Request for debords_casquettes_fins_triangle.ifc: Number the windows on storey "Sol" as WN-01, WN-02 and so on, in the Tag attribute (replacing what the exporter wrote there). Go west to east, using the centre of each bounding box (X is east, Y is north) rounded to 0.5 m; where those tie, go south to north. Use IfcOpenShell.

First a look at what the model holds.

```python
import ifcopenshell
import ifcopenshell.util.element
import ifcopenshell.util.placement

model = ifcopenshell.open("debords_casquettes_fins_triangle.ifc")
print(model.schema)
storey = next(s for s in model.by_type("IfcBuildingStorey") if s.Name == "Sol")
windows = [e for e in ifcopenshell.util.element.get_decomposition(storey) if e.is_a("IfcWindow")]
for e in sorted(windows, key=lambda e: e.id()):
    origin = ifcopenshell.util.placement.get_local_placement(e.ObjectPlacement)[:3, 3]
    print(e.id(), e.Tag, e.Name, origin.round(2) + 0.0, sep=" | ")
```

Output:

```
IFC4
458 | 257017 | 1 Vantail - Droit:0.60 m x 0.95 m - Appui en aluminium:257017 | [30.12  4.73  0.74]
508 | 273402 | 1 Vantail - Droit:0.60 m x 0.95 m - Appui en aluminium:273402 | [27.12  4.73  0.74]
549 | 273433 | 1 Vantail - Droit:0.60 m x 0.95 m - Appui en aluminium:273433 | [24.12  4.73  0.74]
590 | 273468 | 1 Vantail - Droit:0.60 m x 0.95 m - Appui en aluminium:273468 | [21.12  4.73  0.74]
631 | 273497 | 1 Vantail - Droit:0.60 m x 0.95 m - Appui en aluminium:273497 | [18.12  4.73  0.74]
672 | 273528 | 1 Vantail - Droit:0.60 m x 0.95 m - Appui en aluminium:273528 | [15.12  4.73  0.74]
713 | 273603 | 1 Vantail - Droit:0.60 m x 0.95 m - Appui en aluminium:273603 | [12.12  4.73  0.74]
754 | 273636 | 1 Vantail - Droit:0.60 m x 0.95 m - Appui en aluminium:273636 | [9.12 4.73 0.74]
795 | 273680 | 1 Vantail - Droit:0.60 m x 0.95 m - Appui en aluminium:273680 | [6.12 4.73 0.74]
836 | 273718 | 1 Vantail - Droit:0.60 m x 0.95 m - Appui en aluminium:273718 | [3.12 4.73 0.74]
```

```python
import ifcopenshell
import ifcopenshell.geom
import ifcopenshell.util.element
import ifcopenshell.util.shape

model = ifcopenshell.open("debords_casquettes_fins_triangle.ifc")
settings = ifcopenshell.geom.settings()
settings.set("use-world-coords", True)


def centre(element):
    shape = ifcopenshell.geom.create_shape(settings, element)
    return ifcopenshell.util.shape.get_bbox_centroid(shape.geometry)


storey = next(s for s in model.by_type("IfcBuildingStorey") if s.Name == "Sol")
windows = [e for e in ifcopenshell.util.element.get_decomposition(storey) if e.is_a("IfcWindow")]

# Insertion points can sit at a corner or the storey origin, so sort by the geometry (in metres).
centres = {e: centre(e) for e in windows}
windows.sort(key=lambda e: (round(centres[e][0] / 0.5), centres[e][1]))

for i, e in enumerate(windows, start=1):
    number = f"WN-{i:02d}"
    e.Tag = number
    print(e.id(), number)

model.write("debords_casquettes_fins_triangle_v2.ifc")
```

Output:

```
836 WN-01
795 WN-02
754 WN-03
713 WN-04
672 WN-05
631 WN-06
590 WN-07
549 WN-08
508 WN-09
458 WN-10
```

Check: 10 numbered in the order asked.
